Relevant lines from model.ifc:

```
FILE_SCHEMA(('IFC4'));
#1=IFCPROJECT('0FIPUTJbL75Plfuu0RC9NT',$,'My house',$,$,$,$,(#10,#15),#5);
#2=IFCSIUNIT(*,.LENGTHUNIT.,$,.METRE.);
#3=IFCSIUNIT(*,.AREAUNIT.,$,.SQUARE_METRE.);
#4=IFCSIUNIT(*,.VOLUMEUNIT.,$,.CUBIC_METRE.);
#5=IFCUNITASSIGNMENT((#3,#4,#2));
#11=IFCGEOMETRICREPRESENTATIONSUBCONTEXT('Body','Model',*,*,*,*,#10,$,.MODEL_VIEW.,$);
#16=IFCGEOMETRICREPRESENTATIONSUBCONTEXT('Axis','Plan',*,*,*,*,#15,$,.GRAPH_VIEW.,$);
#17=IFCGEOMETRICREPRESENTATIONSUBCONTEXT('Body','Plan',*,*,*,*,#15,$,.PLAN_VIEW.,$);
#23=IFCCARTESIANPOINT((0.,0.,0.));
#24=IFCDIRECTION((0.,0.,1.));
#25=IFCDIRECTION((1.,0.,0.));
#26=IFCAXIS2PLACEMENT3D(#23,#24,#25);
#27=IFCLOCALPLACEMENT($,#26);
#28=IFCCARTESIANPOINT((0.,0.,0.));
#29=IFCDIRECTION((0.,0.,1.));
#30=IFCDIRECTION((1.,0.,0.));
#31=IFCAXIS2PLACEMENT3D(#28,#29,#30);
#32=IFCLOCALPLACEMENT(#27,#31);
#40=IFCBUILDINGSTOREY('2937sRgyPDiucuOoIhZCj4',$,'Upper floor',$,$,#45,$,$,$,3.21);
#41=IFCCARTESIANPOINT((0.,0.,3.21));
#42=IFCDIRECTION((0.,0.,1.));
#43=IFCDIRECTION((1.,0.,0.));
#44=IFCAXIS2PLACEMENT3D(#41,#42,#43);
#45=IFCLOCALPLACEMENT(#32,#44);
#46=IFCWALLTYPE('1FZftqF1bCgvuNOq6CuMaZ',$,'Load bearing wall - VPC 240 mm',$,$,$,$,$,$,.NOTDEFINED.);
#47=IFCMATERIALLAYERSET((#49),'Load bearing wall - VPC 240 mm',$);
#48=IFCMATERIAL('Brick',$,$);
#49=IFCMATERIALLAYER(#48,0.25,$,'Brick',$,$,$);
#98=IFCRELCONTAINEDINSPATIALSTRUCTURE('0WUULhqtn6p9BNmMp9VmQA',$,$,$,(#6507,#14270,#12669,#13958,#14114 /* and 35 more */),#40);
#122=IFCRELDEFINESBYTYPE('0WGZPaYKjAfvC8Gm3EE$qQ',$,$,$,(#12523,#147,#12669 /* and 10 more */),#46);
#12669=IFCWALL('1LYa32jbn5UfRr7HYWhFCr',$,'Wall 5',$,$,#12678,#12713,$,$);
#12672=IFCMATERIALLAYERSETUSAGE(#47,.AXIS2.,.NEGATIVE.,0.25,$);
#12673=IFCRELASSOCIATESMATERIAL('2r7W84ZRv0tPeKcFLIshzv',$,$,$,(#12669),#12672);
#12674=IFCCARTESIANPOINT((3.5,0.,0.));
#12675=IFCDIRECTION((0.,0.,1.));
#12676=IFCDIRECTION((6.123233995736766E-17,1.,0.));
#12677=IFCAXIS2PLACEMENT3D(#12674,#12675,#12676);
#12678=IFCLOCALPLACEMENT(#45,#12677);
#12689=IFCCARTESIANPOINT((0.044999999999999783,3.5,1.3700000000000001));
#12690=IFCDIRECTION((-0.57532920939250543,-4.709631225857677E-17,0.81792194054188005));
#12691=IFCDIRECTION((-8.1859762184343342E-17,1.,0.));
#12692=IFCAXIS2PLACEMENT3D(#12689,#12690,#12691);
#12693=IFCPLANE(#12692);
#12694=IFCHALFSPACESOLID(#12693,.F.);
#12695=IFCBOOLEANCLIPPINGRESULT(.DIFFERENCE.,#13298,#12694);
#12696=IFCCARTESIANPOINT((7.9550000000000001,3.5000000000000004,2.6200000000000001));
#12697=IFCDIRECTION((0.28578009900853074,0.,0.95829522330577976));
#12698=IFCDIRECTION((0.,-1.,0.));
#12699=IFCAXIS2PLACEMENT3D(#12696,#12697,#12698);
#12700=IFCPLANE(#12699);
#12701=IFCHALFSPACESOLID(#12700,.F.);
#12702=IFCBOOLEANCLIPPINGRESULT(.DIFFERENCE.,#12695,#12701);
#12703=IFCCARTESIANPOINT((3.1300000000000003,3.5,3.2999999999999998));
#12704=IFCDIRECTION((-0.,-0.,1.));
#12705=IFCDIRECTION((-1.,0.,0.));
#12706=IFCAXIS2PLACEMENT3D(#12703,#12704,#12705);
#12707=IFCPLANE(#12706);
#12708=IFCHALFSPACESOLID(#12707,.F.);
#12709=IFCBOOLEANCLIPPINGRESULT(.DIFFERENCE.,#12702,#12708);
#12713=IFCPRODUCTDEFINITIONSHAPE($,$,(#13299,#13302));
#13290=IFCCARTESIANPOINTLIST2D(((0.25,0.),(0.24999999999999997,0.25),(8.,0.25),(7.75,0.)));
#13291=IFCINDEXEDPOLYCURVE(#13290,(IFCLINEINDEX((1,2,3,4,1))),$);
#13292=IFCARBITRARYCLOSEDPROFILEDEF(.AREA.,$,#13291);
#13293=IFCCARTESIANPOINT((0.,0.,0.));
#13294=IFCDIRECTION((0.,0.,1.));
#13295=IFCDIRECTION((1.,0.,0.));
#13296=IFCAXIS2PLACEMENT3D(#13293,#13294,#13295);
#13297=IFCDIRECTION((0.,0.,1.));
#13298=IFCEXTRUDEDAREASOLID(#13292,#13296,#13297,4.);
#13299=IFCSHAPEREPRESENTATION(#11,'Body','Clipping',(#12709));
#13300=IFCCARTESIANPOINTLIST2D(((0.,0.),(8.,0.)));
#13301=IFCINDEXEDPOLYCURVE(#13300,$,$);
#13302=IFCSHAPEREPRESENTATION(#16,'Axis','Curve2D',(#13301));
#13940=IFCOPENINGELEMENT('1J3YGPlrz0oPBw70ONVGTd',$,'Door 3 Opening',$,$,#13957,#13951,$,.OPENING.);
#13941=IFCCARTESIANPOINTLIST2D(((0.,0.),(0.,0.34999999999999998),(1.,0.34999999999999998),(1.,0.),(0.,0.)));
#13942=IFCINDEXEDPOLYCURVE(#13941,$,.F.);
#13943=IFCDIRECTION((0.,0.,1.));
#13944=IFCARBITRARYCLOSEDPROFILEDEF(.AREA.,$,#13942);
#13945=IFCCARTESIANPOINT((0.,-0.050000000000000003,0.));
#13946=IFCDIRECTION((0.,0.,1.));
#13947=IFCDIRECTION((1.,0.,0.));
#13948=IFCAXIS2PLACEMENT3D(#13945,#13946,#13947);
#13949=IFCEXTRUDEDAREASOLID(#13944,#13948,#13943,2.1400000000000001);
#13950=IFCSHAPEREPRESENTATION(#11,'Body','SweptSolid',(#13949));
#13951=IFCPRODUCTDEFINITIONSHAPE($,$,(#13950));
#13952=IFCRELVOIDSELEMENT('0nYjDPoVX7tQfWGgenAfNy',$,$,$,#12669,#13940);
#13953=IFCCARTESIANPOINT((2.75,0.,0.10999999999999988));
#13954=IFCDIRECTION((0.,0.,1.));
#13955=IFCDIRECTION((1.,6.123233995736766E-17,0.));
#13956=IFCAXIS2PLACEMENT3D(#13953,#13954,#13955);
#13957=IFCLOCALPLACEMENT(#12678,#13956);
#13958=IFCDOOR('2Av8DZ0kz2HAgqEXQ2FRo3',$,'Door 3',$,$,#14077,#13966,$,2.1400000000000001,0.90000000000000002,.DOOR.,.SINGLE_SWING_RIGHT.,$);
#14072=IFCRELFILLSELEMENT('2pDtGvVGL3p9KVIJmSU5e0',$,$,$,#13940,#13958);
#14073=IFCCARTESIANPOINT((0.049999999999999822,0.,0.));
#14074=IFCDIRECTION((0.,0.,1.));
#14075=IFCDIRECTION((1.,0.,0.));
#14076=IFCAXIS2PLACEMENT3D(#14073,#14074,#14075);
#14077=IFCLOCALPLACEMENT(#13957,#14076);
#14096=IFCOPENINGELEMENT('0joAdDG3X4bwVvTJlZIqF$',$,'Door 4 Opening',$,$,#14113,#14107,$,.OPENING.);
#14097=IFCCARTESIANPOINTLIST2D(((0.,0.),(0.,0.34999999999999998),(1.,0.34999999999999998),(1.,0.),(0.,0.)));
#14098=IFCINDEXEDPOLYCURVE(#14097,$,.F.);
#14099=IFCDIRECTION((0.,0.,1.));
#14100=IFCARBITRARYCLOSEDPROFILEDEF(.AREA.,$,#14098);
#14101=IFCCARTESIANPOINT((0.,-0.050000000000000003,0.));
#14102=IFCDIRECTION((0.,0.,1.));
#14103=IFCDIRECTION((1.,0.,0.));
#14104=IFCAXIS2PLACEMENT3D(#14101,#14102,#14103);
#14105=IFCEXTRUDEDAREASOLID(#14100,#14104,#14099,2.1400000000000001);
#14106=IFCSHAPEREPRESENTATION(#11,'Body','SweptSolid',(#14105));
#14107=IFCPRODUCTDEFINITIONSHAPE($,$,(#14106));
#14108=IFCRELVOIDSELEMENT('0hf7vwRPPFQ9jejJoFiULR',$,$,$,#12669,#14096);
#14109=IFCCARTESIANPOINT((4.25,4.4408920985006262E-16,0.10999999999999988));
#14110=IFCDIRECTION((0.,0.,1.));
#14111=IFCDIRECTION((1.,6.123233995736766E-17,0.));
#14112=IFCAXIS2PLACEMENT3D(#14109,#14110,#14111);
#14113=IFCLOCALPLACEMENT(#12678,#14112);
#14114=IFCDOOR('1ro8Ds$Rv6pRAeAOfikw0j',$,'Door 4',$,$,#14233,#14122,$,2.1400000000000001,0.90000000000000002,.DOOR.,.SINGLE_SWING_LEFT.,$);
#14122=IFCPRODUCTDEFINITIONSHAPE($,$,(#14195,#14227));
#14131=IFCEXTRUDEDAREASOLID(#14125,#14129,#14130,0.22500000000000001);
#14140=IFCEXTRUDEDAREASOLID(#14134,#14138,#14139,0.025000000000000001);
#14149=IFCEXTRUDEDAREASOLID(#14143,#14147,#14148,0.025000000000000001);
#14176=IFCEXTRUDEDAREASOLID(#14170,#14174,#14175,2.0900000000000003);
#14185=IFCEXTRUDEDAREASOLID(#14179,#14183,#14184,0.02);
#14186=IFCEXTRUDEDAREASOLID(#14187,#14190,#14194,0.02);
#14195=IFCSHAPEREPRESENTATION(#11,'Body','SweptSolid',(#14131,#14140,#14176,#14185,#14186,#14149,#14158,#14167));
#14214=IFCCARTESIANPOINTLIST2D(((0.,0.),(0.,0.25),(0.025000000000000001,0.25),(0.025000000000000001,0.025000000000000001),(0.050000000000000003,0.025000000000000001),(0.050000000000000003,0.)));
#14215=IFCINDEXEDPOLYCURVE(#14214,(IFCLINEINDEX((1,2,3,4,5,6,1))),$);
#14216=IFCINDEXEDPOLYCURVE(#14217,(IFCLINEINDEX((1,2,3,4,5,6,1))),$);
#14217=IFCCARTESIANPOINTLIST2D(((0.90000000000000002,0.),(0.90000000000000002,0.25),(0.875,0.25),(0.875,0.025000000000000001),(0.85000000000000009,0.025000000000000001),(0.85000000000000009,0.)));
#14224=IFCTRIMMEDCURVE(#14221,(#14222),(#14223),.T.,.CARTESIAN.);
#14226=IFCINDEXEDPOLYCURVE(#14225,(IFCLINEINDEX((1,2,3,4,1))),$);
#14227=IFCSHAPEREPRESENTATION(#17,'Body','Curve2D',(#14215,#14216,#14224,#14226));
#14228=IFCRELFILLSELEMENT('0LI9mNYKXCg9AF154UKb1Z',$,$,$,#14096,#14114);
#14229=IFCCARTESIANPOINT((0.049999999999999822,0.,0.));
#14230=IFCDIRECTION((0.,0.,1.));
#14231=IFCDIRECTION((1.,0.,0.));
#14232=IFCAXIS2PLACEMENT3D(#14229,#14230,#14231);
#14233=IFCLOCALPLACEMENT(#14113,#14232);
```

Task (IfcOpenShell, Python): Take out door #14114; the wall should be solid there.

```python
import ifcopenshell
import ifcopenshell.api.feature
import ifcopenshell.api.root
import ifcopenshell.geom
import ifcopenshell.util.shape

model = ifcopenshell.open("model.ifc")
settings = ifcopenshell.geom.settings()


def volume(element):
    """Net volume in cubic metres, openings subtracted."""
    shape = ifcopenshell.geom.create_shape(settings, element)
    return ifcopenshell.util.shape.get_volume(shape.geometry)


door = model.by_id(14114)
opening = door.FillsVoids[0].RelatingOpeningElement
wall = opening.VoidsElements[0].RelatingBuildingElement
before = volume(wall)

ifcopenshell.api.root.remove_product(model, product=door)
ifcopenshell.api.feature.remove_feature(model, feature=opening)

after = volume(wall)

print(f"wall volume {before:.3f} -> {after:.3f} m3")

model.write("model_updated.ifc")
```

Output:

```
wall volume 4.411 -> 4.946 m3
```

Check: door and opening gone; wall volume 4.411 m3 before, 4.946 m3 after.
